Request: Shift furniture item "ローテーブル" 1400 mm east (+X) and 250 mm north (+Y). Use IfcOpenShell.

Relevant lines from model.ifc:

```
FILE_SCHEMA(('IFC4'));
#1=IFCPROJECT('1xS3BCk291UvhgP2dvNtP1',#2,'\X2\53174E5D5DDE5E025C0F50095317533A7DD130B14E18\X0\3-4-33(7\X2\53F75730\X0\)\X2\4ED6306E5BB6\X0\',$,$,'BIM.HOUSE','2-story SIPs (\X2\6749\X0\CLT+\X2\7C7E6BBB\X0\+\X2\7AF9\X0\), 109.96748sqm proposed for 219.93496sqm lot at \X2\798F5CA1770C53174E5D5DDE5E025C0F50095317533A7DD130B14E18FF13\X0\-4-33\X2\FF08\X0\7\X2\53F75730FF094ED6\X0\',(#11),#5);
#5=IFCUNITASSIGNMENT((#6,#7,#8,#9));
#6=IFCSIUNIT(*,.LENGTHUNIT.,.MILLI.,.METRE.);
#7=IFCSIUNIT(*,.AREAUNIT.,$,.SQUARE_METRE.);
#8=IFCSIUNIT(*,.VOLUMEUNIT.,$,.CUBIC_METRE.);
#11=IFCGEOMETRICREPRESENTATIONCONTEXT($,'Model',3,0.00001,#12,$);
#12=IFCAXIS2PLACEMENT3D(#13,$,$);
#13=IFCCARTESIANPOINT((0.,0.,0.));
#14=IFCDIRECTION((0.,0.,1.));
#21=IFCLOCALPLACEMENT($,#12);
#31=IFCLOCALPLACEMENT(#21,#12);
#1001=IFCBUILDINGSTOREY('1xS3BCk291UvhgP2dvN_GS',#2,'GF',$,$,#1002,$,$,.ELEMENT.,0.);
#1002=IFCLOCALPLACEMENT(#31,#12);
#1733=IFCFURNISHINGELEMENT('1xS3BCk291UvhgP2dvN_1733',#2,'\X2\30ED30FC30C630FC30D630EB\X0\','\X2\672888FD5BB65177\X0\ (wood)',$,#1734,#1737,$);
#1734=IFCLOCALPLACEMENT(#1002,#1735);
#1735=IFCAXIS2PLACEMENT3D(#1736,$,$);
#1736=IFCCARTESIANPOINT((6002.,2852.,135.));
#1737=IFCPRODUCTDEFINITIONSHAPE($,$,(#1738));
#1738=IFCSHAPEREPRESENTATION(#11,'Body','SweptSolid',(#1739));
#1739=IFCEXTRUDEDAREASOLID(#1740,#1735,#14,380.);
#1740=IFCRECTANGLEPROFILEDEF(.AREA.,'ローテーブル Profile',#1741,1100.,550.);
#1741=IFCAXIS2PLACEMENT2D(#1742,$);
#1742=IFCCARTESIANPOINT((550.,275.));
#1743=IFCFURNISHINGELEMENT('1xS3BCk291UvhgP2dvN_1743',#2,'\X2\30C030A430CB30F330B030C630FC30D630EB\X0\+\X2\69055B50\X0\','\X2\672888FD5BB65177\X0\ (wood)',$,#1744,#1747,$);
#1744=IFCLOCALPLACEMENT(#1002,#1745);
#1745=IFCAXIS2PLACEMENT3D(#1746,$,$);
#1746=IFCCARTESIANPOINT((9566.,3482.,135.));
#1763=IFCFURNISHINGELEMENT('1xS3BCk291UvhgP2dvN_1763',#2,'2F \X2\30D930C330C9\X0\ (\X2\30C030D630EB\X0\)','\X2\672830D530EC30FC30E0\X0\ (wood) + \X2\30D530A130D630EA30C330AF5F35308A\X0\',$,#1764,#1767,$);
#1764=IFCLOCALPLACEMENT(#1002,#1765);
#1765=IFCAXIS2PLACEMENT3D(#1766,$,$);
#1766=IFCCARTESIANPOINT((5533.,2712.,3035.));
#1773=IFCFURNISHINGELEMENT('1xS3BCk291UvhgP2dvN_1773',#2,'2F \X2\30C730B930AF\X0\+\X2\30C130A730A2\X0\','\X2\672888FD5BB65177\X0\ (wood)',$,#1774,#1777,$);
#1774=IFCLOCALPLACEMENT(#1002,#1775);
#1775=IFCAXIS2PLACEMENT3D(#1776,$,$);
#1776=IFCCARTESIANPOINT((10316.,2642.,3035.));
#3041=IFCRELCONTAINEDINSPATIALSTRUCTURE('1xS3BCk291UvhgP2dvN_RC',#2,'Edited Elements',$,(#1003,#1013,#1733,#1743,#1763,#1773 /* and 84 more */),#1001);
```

```python
import ifcopenshell
import ifcopenshell.api.geometry
import ifcopenshell.util.placement
import ifcopenshell.util.unit

model = ifcopenshell.open("model.ifc")
unit_scale = ifcopenshell.util.unit.calculate_unit_scale(model)

item = model.by_guid("1xS3BCk291UvhgP2dvN_1733")
matrix = ifcopenshell.util.placement.get_local_placement(item.ObjectPlacement)
matrix[0, 3] += 1.4 / unit_scale
matrix[1, 3] += 0.25 / unit_scale
ifcopenshell.api.geometry.edit_object_placement(model, product=item, matrix=matrix, is_si=False)

print(ifcopenshell.util.placement.get_local_placement(item.ObjectPlacement).round(3) + 0.0)

model.write("model_rev.ifc")
```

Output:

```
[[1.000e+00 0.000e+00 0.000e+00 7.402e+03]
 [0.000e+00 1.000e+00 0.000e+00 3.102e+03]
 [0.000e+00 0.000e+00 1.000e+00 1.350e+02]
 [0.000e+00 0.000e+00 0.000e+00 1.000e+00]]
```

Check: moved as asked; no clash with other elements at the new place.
